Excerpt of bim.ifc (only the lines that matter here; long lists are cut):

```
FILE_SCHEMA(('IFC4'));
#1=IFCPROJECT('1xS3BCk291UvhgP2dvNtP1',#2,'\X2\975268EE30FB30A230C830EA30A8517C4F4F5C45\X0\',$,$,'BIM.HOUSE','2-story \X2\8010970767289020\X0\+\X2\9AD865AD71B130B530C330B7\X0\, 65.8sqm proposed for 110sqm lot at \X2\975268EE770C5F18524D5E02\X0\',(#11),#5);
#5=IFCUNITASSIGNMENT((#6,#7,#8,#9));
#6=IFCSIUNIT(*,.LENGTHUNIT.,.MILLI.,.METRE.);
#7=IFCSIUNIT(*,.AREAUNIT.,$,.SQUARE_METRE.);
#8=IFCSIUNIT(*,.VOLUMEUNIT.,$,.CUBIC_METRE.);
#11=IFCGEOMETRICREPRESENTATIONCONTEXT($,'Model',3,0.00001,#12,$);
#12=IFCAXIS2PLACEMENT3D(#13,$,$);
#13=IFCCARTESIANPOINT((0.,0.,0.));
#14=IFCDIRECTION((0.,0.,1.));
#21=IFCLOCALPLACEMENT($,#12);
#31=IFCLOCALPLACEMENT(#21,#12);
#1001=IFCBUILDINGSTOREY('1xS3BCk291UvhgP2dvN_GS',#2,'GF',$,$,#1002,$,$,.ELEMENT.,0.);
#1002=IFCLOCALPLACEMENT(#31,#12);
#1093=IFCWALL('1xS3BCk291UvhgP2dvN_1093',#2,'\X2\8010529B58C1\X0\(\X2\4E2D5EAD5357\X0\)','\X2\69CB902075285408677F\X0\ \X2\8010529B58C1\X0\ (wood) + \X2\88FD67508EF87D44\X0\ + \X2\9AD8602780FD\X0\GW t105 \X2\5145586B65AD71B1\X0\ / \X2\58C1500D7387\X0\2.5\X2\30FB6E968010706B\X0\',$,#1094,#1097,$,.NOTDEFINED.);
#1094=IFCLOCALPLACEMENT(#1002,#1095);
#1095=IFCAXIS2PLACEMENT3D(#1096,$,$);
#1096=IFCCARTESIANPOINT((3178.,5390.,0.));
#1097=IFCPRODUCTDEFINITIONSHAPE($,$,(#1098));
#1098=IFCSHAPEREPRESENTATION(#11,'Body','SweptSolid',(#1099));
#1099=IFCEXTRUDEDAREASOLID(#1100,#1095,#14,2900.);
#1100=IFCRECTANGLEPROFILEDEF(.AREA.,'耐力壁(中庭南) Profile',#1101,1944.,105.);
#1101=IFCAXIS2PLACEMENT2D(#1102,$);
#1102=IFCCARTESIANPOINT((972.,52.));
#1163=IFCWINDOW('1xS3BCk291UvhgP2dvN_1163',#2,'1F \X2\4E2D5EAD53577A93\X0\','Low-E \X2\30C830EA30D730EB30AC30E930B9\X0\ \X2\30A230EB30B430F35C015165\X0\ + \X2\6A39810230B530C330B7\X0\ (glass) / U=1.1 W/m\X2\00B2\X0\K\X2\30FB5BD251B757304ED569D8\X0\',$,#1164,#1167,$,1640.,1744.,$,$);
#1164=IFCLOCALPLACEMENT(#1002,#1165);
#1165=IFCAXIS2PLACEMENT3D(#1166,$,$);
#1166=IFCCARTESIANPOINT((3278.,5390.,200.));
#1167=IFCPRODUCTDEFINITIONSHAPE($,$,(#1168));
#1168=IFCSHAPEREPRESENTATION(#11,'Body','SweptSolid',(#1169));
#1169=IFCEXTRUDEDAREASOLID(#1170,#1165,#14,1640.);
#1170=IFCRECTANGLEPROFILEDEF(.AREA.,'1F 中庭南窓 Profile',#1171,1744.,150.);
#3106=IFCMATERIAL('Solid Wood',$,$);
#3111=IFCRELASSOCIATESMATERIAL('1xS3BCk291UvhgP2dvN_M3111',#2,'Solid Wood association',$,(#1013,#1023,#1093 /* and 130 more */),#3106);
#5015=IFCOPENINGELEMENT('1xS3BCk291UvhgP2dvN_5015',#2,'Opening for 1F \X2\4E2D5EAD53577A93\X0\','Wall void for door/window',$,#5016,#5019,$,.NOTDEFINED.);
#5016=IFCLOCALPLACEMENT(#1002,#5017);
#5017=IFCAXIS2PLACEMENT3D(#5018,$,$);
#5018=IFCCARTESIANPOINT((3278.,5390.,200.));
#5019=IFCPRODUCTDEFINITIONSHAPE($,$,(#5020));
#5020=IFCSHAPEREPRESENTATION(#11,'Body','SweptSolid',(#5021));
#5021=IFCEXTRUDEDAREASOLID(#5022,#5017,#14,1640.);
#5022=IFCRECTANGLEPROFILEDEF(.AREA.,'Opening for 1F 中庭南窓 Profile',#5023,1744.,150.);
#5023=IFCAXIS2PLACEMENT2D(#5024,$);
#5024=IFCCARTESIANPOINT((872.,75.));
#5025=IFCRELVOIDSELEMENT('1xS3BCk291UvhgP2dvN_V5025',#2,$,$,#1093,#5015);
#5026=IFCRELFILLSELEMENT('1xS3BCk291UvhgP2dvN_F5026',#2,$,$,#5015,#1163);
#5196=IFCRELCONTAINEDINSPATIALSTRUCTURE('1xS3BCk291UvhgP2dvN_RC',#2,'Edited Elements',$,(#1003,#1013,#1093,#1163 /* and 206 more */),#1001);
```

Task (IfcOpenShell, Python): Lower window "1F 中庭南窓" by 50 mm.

```python
import numpy as np
import ifcopenshell
import ifcopenshell.api.geometry
import ifcopenshell.util.placement
import ifcopenshell.util.unit

model = ifcopenshell.open("bim.ifc")
unit_scale = ifcopenshell.util.unit.calculate_unit_scale(model)

window = model.by_guid("1xS3BCk291UvhgP2dvN_1163")
opening = window.FillsVoids[0].RelatingOpeningElement
dz = -0.05 / unit_scale

shift = np.array([0.0, 0.0, dz])
# The window is not placed relative to its opening, so move both.
for product in (opening, window):
    matrix = ifcopenshell.util.placement.get_local_placement(product.ObjectPlacement)
    matrix[:3, 3] += shift
    ifcopenshell.api.geometry.edit_object_placement(model, product=product, matrix=matrix, is_si=False)

print(f"moved by {dz * unit_scale:+.3f} m")

model.write("bim_updated.ifc")
```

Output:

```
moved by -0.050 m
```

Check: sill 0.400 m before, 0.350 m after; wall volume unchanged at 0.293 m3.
